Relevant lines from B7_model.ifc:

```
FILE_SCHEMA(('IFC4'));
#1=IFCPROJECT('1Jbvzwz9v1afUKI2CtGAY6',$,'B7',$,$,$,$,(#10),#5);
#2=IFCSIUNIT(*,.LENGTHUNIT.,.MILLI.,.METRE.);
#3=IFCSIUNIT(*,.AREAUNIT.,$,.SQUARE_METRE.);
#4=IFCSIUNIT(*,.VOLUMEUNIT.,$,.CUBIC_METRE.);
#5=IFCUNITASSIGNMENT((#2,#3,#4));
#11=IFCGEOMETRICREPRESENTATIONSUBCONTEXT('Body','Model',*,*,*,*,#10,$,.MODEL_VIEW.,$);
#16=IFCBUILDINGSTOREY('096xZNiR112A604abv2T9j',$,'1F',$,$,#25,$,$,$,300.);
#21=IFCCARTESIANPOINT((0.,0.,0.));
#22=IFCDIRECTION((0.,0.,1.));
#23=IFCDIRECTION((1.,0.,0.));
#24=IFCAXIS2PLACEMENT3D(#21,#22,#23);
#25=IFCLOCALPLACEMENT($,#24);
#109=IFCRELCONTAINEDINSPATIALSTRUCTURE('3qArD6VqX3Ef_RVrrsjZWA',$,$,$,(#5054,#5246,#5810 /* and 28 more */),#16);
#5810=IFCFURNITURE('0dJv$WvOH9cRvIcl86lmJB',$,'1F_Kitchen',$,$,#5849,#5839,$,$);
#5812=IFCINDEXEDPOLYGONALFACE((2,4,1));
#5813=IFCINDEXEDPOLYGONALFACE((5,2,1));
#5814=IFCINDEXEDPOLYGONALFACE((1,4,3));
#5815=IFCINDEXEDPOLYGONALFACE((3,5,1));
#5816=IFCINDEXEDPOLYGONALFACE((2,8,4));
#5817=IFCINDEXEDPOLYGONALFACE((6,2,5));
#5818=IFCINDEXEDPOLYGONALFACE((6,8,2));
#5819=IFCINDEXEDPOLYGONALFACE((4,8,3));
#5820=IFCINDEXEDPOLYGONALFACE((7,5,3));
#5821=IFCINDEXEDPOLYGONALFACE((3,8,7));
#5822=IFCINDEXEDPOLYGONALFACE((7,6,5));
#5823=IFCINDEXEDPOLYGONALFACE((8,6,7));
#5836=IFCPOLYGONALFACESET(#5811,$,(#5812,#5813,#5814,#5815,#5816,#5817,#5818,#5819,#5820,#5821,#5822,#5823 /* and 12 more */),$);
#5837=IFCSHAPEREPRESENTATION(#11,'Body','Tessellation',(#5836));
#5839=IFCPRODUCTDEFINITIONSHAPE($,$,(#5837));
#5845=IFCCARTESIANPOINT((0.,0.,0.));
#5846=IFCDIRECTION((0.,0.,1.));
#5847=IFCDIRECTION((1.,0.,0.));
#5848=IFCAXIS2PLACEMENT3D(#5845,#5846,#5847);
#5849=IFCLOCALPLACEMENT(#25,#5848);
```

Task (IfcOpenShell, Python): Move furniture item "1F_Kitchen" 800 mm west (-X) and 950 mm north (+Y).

```python
import ifcopenshell
import ifcopenshell.api.geometry
import ifcopenshell.util.placement
import ifcopenshell.util.unit

model = ifcopenshell.open("B7_model.ifc")
unit_scale = ifcopenshell.util.unit.calculate_unit_scale(model)

item = model.by_guid("0dJv$WvOH9cRvIcl86lmJB")
matrix = ifcopenshell.util.placement.get_local_placement(item.ObjectPlacement)
matrix[0, 3] -= 0.8 / unit_scale
matrix[1, 3] += 0.95 / unit_scale
ifcopenshell.api.geometry.edit_object_placement(model, product=item, matrix=matrix, is_si=False)

print(ifcopenshell.util.placement.get_local_placement(item.ObjectPlacement).round(3) + 0.0)

model.write("B7_model_v2.ifc")
```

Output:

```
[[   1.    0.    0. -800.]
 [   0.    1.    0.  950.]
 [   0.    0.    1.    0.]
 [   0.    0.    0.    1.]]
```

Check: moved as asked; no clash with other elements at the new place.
